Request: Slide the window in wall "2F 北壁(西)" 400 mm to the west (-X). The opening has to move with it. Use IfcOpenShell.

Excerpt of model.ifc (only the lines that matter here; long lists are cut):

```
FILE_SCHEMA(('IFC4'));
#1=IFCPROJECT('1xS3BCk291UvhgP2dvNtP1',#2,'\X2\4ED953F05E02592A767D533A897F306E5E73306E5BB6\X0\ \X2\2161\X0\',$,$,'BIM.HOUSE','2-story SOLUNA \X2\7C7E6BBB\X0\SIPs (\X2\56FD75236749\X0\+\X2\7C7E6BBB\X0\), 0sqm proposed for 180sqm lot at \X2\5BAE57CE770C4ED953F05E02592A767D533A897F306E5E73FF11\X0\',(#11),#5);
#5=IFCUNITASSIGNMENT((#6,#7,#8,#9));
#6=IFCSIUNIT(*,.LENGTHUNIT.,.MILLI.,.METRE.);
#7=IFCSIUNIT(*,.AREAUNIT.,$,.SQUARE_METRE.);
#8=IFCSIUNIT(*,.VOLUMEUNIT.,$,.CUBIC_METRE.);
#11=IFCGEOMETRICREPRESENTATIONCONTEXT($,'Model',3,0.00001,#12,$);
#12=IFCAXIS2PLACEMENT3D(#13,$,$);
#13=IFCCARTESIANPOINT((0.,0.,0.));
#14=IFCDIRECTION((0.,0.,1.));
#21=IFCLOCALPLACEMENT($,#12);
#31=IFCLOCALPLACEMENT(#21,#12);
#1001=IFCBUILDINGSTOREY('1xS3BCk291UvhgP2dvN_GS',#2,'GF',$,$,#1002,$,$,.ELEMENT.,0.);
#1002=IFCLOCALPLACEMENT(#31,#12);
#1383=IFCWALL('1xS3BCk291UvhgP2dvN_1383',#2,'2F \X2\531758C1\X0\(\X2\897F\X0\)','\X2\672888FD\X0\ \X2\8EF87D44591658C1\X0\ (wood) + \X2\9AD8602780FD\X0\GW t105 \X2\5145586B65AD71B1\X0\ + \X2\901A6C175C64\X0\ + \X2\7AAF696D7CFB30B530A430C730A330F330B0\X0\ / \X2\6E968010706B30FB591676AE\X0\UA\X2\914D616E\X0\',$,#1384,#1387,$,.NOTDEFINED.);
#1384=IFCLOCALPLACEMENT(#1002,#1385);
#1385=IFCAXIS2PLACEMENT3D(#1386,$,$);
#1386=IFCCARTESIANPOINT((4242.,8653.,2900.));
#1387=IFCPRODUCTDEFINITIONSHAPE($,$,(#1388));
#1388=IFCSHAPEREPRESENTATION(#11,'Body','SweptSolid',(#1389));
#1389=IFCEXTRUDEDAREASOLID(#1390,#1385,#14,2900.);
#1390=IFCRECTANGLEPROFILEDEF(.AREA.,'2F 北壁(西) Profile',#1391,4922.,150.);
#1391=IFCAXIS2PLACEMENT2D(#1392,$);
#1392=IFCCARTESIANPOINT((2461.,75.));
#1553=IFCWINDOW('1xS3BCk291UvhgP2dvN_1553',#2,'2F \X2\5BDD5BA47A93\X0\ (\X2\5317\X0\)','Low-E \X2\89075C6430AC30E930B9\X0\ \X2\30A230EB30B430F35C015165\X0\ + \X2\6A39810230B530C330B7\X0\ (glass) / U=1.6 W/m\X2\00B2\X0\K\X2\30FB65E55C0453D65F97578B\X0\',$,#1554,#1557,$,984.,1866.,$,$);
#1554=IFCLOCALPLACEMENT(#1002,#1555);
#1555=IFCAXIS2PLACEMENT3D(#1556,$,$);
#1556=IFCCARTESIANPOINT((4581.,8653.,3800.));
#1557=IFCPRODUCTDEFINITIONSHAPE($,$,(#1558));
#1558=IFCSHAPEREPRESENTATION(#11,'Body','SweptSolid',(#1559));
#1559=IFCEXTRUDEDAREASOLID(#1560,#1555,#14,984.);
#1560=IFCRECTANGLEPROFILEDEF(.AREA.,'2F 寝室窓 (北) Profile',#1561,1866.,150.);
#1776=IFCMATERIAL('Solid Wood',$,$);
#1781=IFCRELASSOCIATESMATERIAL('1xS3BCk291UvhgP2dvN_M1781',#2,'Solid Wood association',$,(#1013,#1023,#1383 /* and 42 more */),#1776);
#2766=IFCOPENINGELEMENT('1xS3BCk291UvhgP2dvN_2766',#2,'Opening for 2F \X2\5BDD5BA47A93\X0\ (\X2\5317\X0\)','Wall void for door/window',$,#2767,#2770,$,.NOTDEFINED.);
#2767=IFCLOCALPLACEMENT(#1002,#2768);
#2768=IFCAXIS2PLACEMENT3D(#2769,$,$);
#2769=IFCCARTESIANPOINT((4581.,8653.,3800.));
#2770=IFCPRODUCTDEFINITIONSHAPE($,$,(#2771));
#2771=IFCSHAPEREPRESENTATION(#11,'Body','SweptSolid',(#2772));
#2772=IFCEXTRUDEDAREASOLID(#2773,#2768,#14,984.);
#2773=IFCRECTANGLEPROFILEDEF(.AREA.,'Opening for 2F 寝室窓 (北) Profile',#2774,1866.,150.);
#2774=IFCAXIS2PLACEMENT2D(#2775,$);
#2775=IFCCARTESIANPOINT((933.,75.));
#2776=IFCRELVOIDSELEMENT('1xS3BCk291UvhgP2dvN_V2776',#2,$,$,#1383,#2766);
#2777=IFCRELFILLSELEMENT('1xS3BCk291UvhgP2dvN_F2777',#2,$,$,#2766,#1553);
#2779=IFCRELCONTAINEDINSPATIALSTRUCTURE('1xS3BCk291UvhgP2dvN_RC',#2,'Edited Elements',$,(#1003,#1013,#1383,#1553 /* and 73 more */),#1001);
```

```python
import ifcopenshell
import ifcopenshell.api.geometry
import ifcopenshell.util.placement

model = ifcopenshell.open("model.ifc")

window = model.by_id(1553)
opening = window.FillsVoids[0].RelatingOpeningElement
wall = opening.VoidsElements[0].RelatingBuildingElement

wall_matrix = ifcopenshell.util.placement.get_local_placement(wall.ObjectPlacement)
shift = wall_matrix[:3, 0] * -400.0
before = ifcopenshell.util.placement.get_local_placement(window.ObjectPlacement)[:3, 3].copy()

# The window is not placed relative to its opening, so move both.
for product in (opening, window):
    matrix = ifcopenshell.util.placement.get_local_placement(product.ObjectPlacement)
    matrix[:3, 3] += shift
    ifcopenshell.api.geometry.edit_object_placement(model, product=product, matrix=matrix, is_si=False)

after = ifcopenshell.util.placement.get_local_placement(window.ObjectPlacement)[:3, 3]
print("window moved by", (after - before).round(3) + 0.0)

model.write("model_rev.ifc")
```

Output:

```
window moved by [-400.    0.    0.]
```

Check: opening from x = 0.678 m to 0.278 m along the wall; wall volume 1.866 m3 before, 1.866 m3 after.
